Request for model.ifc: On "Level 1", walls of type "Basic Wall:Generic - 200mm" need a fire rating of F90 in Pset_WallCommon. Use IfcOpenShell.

First a look at what the model holds.

```python
import ifcopenshell
import ifcopenshell.util.element

model = ifcopenshell.open("model.ifc")
print(model.schema)
storey = next(s for s in model.by_type("IfcBuildingStorey") if s.Name == "Level 1")
walls = [e for e in ifcopenshell.util.element.get_decomposition(storey) if e.is_a("IfcWall")]
seen = {}
for e in walls:
    element_type = ifcopenshell.util.element.get_type(e)
    key = (element_type.Name if element_type != e and element_type else None, ifcopenshell.util.element.get_pset(e, "Pset_WallCommon", "FireRating"))
    seen[key] = seen.get(key, 0) + 1
for (name, value), count in sorted(seen.items(), key=str):
    print(count, "x", name, "|", value)
```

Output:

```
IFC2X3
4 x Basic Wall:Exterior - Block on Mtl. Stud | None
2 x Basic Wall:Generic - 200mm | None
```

```python
import ifcopenshell
import ifcopenshell.api.pset
import ifcopenshell.util.element

model = ifcopenshell.open("model.ifc")

storey = next(s for s in model.by_type("IfcBuildingStorey") if s.Name == "Level 1")
walls = [e for e in ifcopenshell.util.element.get_decomposition(storey) if e.is_a("IfcWall")]

count = 0
for e in walls:
    element_type = ifcopenshell.util.element.get_type(e)
    if element_type in (None, e) or element_type.Name != "Basic Wall:Generic - 200mm":
        continue
    # add_pset returns the element's existing set when there is one.
    pset = ifcopenshell.api.pset.add_pset(model, product=e, name="Pset_WallCommon")
    ifcopenshell.api.pset.edit_pset(model, pset=pset, properties={"FireRating": "F90"})
    count += 1

print(count, "walls updated")

model.write("model-out.ifc")
```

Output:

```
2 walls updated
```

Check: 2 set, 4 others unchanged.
